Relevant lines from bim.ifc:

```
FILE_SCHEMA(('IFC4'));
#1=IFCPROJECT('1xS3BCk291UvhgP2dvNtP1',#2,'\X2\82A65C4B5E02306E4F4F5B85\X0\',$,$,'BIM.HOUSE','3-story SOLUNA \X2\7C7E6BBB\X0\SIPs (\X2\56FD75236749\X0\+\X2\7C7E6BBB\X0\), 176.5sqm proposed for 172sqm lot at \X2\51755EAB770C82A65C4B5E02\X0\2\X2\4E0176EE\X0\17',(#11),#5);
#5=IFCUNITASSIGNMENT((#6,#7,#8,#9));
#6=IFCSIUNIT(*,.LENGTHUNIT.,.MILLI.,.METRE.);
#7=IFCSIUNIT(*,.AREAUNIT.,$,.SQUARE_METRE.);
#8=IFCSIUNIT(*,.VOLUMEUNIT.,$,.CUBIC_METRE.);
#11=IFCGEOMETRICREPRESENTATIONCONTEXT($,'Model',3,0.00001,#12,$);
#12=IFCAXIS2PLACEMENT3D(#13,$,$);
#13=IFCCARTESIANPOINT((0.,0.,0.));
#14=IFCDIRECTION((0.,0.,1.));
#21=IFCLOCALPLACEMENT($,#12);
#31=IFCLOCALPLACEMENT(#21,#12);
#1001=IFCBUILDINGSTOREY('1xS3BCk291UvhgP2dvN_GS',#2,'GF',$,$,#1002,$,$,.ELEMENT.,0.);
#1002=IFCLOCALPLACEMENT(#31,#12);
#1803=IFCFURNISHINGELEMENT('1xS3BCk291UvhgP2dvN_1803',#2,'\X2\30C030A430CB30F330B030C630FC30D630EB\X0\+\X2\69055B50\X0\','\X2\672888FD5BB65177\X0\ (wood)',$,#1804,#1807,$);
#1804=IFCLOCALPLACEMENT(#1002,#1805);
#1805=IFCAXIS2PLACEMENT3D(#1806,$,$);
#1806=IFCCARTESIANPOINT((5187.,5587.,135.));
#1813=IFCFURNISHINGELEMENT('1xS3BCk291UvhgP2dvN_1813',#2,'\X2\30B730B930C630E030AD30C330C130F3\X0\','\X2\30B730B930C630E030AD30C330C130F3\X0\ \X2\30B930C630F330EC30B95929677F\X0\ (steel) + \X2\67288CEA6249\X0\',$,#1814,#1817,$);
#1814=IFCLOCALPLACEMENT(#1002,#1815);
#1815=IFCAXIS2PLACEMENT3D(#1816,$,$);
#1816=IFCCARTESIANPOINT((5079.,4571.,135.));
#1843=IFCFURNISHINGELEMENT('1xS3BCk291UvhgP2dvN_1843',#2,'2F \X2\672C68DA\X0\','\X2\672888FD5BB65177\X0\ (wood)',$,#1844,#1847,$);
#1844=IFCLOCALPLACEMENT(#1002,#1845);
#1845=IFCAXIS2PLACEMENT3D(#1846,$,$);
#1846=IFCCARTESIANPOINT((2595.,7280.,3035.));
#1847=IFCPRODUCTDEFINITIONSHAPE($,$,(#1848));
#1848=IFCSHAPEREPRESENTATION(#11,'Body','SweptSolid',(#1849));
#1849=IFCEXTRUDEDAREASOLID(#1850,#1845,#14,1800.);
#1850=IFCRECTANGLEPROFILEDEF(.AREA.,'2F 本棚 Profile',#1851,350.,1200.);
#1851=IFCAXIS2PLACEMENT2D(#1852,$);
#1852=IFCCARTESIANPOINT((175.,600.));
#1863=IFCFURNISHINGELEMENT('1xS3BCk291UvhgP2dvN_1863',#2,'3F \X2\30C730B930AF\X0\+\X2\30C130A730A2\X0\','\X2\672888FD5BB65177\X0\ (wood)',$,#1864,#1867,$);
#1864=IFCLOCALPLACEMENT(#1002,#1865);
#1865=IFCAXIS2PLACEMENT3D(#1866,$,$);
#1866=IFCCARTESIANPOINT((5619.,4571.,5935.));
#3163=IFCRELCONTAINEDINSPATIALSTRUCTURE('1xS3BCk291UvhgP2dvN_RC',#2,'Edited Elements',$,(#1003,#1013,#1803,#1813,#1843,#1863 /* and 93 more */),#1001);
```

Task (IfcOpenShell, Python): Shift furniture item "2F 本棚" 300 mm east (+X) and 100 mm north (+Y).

```python
import ifcopenshell
import ifcopenshell.api.geometry
import ifcopenshell.util.placement
import ifcopenshell.util.unit

model = ifcopenshell.open("bim.ifc")
unit_scale = ifcopenshell.util.unit.calculate_unit_scale(model)

item = model.by_id(1843)
matrix = ifcopenshell.util.placement.get_local_placement(item.ObjectPlacement)
matrix[0, 3] += 0.3 / unit_scale
matrix[1, 3] += 0.1 / unit_scale
ifcopenshell.api.geometry.edit_object_placement(model, product=item, matrix=matrix, is_si=False)

print(ifcopenshell.util.placement.get_local_placement(item.ObjectPlacement).round(3) + 0.0)

model.write("bim_v2.ifc")
```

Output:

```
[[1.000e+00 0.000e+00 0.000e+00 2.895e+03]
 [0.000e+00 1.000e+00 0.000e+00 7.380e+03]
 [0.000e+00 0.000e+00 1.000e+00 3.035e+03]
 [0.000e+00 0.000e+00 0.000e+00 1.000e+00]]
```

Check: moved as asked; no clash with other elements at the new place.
